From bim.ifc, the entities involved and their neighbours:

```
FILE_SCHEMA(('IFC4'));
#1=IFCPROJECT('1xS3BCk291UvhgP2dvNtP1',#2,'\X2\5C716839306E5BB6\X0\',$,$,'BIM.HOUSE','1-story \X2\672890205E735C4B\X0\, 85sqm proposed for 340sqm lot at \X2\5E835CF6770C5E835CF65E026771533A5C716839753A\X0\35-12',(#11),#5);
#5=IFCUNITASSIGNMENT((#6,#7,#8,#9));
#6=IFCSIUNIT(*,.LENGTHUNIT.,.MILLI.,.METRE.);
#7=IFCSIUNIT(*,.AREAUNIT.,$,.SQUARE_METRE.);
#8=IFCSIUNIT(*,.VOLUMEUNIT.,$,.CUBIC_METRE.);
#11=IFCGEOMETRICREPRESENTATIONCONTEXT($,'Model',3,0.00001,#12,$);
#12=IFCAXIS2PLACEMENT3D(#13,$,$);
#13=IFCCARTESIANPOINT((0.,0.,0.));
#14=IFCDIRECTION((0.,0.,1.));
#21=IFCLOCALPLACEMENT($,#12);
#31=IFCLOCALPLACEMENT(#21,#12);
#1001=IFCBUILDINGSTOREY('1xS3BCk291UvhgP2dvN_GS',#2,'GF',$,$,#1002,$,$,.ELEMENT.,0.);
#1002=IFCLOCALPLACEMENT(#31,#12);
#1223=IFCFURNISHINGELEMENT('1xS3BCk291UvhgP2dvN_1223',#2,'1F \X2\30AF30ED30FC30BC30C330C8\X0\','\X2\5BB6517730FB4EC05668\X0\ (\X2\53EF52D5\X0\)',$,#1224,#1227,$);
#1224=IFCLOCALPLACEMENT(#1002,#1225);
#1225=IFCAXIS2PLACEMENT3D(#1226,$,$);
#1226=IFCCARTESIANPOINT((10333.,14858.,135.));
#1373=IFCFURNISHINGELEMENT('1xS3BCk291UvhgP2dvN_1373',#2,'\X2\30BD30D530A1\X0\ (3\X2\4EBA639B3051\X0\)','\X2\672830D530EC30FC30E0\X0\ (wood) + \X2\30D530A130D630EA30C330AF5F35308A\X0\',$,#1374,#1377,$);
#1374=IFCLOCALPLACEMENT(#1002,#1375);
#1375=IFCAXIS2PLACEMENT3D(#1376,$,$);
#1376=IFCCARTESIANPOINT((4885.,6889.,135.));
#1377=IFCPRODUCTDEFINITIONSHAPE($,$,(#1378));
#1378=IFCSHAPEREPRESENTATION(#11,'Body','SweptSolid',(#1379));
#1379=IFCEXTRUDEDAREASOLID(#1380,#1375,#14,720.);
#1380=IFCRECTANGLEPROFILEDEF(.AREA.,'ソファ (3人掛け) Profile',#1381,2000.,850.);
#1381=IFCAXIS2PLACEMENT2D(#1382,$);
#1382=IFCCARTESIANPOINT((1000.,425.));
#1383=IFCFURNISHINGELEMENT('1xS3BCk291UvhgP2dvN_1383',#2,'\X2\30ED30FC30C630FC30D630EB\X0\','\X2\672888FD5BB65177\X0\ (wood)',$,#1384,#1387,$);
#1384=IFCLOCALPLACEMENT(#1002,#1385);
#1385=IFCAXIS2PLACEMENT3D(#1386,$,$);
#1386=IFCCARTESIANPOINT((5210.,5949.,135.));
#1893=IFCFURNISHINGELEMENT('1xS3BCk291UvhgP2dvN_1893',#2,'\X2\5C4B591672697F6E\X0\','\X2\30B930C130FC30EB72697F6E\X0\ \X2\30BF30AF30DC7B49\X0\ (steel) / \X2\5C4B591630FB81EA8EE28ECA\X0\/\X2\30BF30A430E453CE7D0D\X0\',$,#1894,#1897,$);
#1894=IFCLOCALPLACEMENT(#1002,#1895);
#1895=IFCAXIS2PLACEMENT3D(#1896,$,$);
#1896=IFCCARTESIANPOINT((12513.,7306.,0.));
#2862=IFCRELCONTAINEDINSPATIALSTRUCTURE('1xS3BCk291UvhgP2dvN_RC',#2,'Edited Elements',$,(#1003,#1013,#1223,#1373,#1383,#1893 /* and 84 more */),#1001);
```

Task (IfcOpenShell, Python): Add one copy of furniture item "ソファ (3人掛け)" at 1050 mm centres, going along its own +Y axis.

```python
import ifcopenshell
import ifcopenshell.api.geometry
import ifcopenshell.api.root
import ifcopenshell.util.element
import ifcopenshell.util.placement

model = ifcopenshell.open("bim.ifc")


def reuse_history(source, copy):
    """copy_class also copies each property set's owner history, people and application; keep the originals."""
    for rel in copy.IsDefinedBy:
        if rel.is_a("IfcRelDefinesByProperties") and (history := rel.RelatingPropertyDefinition.OwnerHistory):
            rel.RelatingPropertyDefinition.OwnerHistory = source.OwnerHistory
            ifcopenshell.util.element.remove_deep2(model, history)


source = model.by_guid("1xS3BCk291UvhgP2dvN_1373")
base = ifcopenshell.util.placement.get_local_placement(source.ObjectPlacement)
step = base[:3, 1] * 1050.0

for i in range(1, 2):
    copy = ifcopenshell.api.root.copy_class(model, product=source)
    copy.Representation = ifcopenshell.util.element.copy_deep(
        model, source.Representation, exclude=["IfcGeometricRepresentationContext", "IfcRepresentationMap"]
    )
    reuse_history(source, copy)
    matrix = base.copy()
    matrix[:3, 3] += i * step
    print("added at", matrix[:3, 3].round(3) + 0.0)
    ifcopenshell.api.geometry.edit_object_placement(model, product=copy, matrix=matrix, is_si=False)

model.write("bim_edited.ifc")
```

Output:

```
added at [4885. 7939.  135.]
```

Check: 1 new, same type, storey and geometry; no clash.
